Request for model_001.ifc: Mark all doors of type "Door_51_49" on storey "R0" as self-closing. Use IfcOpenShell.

First a look at what the model holds.

```python
import ifcopenshell
import ifcopenshell.util.element

model = ifcopenshell.open("model_001.ifc")
print(model.schema)
storey = next(s for s in model.by_type("IfcBuildingStorey") if s.Name == "R0")
doors = [e for e in ifcopenshell.util.element.get_decomposition(storey) if e.is_a("IfcDoor")]
seen = {}
for e in doors:
    element_type = ifcopenshell.util.element.get_type(e)
    key = (element_type.Name if element_type != e and element_type else None, ifcopenshell.util.element.get_pset(e, "Pset_DoorCommon", "SelfClosing"))
    seen[key] = seen.get(key, 0) + 1
for (name, value), count in sorted(seen.items(), key=str):
    print(count, "x", name, "|", value)
```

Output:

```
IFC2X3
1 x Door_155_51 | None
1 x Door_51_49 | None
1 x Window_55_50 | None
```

```python
import ifcopenshell
import ifcopenshell.api.pset
import ifcopenshell.util.element

model = ifcopenshell.open("model_001.ifc")

storey = next(s for s in model.by_type("IfcBuildingStorey") if s.Name == "R0")
doors = [e for e in ifcopenshell.util.element.get_decomposition(storey) if e.is_a("IfcDoor")]

count = 0
for e in doors:
    element_type = ifcopenshell.util.element.get_type(e)
    if element_type in (None, e) or element_type.Name != "Door_51_49":
        continue
    # add_pset returns the element's existing set when there is one.
    pset = ifcopenshell.api.pset.add_pset(model, product=e, name="Pset_DoorCommon")
    ifcopenshell.api.pset.edit_pset(model, pset=pset, properties={"SelfClosing": True})
    count += 1

print(count, "doors updated")

model.write("model_001_updated.ifc")
```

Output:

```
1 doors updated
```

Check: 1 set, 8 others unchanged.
